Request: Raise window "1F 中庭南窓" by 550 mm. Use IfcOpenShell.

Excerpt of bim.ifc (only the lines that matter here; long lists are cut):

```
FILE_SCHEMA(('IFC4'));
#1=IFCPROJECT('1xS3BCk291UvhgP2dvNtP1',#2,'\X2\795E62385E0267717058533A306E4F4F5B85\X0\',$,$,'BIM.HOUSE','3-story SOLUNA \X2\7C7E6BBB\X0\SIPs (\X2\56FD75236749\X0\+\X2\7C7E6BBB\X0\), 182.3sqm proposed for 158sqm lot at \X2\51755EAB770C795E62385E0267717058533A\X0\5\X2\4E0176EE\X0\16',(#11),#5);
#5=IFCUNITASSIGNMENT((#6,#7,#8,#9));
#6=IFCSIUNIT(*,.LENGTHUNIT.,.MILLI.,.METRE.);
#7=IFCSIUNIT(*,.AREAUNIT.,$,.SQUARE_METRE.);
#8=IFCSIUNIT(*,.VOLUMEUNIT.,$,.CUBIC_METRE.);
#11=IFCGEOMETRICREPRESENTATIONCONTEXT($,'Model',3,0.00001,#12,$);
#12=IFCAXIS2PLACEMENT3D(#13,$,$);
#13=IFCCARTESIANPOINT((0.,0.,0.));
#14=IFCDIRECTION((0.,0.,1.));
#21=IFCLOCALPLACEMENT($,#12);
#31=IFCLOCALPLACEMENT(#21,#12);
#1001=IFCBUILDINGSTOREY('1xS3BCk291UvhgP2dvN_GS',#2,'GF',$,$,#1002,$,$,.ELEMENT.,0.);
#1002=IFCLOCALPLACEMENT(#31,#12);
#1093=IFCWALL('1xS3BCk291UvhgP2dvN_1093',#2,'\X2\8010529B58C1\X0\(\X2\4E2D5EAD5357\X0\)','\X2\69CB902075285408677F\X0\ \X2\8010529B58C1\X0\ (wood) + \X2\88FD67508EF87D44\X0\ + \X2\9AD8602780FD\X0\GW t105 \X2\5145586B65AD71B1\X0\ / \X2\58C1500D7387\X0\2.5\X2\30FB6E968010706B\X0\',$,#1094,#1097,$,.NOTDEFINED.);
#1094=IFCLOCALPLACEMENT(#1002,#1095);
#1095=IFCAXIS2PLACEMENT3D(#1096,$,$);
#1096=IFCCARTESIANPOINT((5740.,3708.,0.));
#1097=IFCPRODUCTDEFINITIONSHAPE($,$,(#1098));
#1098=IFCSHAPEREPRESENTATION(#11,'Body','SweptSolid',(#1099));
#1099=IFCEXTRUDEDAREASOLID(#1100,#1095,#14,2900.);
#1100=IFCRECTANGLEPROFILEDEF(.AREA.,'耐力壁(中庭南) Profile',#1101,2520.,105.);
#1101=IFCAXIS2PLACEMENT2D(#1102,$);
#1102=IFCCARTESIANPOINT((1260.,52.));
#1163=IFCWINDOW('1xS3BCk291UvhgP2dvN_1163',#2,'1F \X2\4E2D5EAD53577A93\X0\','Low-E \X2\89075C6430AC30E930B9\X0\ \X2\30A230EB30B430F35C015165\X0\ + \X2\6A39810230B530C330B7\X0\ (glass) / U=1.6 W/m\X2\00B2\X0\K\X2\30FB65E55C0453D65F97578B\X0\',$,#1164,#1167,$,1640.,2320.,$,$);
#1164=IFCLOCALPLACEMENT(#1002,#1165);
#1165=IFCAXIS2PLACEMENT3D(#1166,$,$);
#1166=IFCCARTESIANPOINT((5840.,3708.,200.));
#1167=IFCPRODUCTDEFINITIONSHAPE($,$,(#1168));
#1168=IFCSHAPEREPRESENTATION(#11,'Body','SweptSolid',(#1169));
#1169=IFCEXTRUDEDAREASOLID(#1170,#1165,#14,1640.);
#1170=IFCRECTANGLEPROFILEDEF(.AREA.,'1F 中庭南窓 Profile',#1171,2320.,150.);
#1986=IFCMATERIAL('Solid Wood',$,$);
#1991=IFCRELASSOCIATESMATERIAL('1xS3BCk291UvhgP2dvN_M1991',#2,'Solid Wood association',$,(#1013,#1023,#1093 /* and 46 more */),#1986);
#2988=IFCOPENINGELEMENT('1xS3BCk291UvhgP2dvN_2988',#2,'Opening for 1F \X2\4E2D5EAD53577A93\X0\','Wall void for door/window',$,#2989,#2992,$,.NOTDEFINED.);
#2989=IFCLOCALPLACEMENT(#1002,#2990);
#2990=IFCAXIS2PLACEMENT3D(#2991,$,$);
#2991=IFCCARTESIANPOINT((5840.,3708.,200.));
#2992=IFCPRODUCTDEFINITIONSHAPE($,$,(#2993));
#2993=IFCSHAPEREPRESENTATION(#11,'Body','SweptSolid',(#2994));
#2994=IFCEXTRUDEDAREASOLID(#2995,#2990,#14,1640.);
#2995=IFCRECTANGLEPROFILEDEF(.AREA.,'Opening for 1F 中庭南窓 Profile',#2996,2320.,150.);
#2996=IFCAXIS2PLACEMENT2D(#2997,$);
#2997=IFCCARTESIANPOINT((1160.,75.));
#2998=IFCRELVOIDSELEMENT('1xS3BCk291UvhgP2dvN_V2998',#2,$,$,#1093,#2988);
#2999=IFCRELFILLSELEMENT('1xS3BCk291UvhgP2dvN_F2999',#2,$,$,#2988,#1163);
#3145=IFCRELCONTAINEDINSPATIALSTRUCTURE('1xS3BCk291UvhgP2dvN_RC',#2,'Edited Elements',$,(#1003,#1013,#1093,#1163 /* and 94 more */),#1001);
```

```python
import numpy as np
import ifcopenshell
import ifcopenshell.api.geometry
import ifcopenshell.util.placement
import ifcopenshell.util.unit

model = ifcopenshell.open("bim.ifc")
unit_scale = ifcopenshell.util.unit.calculate_unit_scale(model)

window = model.by_guid("1xS3BCk291UvhgP2dvN_1163")
opening = window.FillsVoids[0].RelatingOpeningElement
dz = 0.55 / unit_scale

shift = np.array([0.0, 0.0, dz])
# The window is not placed relative to its opening, so move both.
for product in (opening, window):
    matrix = ifcopenshell.util.placement.get_local_placement(product.ObjectPlacement)
    matrix[:3, 3] += shift
    ifcopenshell.api.geometry.edit_object_placement(model, product=product, matrix=matrix, is_si=False)

print(f"moved by {dz * unit_scale:+.3f} m")

model.write("bim_updated.ifc")
```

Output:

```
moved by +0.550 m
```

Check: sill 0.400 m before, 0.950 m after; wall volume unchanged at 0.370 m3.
